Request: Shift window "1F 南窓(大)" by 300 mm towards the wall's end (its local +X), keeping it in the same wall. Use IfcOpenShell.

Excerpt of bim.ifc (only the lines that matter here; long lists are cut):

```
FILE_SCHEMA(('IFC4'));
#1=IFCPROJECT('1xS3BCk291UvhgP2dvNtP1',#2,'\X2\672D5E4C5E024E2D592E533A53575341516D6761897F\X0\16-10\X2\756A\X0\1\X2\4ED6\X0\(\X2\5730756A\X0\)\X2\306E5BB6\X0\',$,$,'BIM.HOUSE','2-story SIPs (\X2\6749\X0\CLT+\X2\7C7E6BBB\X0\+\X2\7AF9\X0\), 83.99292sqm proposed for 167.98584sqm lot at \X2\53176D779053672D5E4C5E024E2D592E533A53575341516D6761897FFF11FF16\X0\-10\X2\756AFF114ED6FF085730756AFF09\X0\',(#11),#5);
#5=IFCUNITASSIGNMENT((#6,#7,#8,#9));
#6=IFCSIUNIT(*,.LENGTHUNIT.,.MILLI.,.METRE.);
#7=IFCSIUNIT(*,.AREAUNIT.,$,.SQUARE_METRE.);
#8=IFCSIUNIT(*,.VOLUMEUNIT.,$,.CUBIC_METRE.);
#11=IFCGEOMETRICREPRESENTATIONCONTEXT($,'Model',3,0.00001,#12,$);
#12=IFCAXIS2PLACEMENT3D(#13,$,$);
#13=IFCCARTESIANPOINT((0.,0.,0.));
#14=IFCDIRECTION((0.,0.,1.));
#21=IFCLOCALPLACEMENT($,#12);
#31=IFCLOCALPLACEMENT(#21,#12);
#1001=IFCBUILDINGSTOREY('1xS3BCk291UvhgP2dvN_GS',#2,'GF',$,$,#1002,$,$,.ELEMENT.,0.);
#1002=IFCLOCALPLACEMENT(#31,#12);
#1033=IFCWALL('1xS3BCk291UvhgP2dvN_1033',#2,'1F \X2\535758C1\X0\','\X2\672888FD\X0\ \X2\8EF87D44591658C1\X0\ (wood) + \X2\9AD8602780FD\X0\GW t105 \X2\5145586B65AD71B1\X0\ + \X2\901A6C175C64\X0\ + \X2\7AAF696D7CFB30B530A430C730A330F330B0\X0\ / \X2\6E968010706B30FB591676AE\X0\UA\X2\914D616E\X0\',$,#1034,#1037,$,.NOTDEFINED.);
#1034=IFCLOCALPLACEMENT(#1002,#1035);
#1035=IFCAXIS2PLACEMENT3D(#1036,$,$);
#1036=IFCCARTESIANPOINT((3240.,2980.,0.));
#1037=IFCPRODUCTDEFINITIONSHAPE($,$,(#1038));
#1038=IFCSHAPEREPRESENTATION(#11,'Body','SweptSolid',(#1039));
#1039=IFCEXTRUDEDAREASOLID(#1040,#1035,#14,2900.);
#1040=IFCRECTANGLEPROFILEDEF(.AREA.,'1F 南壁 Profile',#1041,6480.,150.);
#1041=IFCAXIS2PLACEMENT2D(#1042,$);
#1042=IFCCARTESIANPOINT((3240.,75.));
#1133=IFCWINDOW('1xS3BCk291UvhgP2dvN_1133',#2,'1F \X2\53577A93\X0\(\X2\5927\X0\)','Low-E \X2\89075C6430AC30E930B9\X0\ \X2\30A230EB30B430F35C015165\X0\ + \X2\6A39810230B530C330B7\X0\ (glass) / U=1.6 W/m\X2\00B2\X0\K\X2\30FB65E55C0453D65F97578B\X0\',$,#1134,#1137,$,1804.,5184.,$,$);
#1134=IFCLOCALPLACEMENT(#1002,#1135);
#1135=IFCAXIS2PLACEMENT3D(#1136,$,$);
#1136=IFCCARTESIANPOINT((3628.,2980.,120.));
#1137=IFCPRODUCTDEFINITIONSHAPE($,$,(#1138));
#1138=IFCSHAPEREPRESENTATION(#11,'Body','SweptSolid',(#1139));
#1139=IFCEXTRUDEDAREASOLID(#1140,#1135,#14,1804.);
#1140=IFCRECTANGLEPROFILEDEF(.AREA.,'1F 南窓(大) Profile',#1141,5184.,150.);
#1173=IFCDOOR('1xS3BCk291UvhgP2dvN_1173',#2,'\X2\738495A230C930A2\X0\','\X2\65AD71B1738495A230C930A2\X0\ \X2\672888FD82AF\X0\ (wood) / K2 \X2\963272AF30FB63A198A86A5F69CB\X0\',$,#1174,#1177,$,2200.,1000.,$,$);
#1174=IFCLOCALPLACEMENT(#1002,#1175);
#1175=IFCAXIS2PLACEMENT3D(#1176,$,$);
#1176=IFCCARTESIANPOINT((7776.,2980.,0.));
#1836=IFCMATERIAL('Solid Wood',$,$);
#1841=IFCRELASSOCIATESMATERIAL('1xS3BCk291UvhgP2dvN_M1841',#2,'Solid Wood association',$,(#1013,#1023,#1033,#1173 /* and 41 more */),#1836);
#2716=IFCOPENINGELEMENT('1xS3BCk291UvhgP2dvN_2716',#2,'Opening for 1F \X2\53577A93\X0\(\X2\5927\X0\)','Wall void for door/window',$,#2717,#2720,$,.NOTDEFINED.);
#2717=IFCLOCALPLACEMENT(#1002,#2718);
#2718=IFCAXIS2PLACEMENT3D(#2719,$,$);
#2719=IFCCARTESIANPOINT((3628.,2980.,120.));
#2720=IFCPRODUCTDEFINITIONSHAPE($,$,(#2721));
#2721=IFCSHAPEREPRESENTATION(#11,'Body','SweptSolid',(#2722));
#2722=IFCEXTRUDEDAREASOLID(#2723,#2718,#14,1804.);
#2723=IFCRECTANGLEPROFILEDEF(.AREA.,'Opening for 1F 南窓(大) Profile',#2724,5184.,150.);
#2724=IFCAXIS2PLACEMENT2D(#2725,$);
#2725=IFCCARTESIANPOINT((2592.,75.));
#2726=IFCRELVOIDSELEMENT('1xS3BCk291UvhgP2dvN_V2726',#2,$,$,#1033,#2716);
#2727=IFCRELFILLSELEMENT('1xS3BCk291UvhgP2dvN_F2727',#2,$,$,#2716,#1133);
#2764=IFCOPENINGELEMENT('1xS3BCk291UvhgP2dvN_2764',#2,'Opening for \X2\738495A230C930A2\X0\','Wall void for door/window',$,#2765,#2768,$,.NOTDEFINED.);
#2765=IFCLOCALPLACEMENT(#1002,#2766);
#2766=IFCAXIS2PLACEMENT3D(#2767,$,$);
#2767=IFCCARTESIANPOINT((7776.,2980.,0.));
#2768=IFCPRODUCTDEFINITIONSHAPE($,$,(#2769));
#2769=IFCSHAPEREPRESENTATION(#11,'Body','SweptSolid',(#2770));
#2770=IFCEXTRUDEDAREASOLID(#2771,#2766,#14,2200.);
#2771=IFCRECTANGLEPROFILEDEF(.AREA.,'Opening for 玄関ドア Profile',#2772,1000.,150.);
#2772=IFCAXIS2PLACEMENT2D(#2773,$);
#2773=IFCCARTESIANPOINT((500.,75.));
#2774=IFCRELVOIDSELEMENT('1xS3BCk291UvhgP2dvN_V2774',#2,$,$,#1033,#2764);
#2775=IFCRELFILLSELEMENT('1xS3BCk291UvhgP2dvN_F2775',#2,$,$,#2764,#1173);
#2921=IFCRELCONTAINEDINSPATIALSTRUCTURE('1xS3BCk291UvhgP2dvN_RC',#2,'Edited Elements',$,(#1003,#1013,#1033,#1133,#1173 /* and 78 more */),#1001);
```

```python
import ifcopenshell
import ifcopenshell.api.geometry
import ifcopenshell.util.placement

model = ifcopenshell.open("bim.ifc")

window = model.by_guid("1xS3BCk291UvhgP2dvN_1133")
opening = window.FillsVoids[0].RelatingOpeningElement
wall = opening.VoidsElements[0].RelatingBuildingElement

wall_matrix = ifcopenshell.util.placement.get_local_placement(wall.ObjectPlacement)
shift = wall_matrix[:3, 0] * 300.0
before = ifcopenshell.util.placement.get_local_placement(window.ObjectPlacement)[:3, 3].copy()

# The window is not placed relative to its opening, so move both.
for product in (opening, window):
    matrix = ifcopenshell.util.placement.get_local_placement(product.ObjectPlacement)
    matrix[:3, 3] += shift
    ifcopenshell.api.geometry.edit_object_placement(model, product=product, matrix=matrix, is_si=False)

after = ifcopenshell.util.placement.get_local_placement(window.ObjectPlacement)[:3, 3]
print("window moved by", (after - before).round(3) + 0.0)

model.write("bim_v2.ifc")
```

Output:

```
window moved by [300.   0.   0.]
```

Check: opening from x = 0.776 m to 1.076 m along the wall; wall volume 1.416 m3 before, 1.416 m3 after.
